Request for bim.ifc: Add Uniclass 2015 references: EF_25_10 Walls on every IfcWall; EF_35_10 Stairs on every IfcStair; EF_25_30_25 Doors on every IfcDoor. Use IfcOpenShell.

First a look at what the model holds.

```python
import ifcopenshell

model = ifcopenshell.open("bim.ifc")
print(model.schema)
print("classifications:", [c.Name for c in model.by_type("IfcClassification")])
for ifc_class in ("IfcDoor", "IfcRoof", "IfcStair", "IfcWall", "IfcWindow"):
    print(ifc_class, len(model.by_type(ifc_class)))
```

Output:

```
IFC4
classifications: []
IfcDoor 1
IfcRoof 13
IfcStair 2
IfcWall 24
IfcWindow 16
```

```python
import ifcopenshell
import ifcopenshell.api.classification

model = ifcopenshell.open("bim.ifc")

system = ifcopenshell.api.classification.add_classification(model, classification="Uniclass 2015")

codes = {
    "IfcWall": ("EF_25_10", "Walls"),
    "IfcStair": ("EF_35_10", "Stairs"),
    "IfcDoor": ("EF_25_30_25", "Doors"),
}
for ifc_class, (code, name) in codes.items():
    products = model.by_type(ifc_class)
    ifcopenshell.api.classification.add_reference(
        model, products=products, classification=system, identification=code, name=name
    )
    print(code, len(products))

model.write("bim_edited.ifc")
```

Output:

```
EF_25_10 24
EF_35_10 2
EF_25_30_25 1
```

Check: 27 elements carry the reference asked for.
